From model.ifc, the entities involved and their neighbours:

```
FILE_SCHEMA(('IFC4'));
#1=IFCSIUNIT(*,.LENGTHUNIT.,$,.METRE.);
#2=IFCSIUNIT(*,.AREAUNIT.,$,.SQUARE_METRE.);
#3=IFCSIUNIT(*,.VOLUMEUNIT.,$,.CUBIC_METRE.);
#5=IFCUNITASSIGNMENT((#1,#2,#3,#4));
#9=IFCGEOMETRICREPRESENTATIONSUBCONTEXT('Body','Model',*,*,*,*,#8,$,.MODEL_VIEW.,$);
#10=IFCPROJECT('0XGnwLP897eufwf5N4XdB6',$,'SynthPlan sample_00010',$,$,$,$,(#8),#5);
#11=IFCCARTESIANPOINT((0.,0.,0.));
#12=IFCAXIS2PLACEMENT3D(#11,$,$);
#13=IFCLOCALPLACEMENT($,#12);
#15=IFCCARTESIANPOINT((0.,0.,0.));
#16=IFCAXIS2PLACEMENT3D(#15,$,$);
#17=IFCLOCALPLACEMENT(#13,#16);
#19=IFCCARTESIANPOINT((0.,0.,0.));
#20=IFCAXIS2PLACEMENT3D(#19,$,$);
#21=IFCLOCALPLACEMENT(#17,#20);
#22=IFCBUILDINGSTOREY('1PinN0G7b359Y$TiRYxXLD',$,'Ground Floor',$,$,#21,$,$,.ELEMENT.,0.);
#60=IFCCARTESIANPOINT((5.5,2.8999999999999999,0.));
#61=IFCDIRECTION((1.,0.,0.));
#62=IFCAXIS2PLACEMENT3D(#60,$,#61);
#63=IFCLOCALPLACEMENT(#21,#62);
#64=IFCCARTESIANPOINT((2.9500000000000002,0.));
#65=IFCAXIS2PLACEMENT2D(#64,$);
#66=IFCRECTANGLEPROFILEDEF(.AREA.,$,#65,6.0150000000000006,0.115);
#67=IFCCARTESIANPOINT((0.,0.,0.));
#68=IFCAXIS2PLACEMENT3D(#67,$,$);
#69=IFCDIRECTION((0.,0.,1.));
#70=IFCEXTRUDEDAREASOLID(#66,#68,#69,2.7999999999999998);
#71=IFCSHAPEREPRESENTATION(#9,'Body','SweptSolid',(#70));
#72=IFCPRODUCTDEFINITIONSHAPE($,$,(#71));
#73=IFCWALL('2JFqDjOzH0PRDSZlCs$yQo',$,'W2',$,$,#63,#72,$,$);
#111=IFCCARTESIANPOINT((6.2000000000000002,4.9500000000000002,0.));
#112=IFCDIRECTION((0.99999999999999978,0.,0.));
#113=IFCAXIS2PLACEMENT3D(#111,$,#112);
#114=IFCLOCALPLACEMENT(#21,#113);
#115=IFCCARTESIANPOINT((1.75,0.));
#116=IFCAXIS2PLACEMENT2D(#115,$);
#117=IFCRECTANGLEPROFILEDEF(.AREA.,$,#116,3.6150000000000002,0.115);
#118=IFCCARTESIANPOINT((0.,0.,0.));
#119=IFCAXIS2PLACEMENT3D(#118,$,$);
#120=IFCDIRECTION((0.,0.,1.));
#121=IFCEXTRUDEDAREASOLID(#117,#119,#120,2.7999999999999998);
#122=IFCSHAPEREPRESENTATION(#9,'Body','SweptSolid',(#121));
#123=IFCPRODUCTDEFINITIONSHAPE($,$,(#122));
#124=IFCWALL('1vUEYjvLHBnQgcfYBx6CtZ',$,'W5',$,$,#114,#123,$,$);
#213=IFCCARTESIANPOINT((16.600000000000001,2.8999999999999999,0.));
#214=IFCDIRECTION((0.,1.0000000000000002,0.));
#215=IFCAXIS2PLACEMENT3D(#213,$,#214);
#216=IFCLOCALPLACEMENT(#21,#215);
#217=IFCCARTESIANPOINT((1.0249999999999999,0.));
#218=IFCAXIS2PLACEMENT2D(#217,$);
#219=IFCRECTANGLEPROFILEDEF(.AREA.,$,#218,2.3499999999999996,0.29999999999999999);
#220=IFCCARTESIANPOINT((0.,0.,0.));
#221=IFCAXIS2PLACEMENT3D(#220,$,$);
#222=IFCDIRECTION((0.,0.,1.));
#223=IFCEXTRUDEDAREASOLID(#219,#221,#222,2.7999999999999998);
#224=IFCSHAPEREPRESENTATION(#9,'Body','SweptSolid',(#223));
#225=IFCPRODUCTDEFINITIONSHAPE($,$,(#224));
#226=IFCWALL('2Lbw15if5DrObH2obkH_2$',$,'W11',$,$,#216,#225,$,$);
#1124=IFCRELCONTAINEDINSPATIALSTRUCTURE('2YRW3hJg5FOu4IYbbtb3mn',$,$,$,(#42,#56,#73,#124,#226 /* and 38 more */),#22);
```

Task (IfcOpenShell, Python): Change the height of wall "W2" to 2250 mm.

```python
import ifcopenshell
import ifcopenshell.geom
import ifcopenshell.util.representation
import ifcopenshell.util.shape
import ifcopenshell.util.unit

model = ifcopenshell.open("model.ifc")
unit_scale = ifcopenshell.util.unit.calculate_unit_scale(model)
settings = ifcopenshell.geom.settings()


def volume(element):
    """Net volume in cubic metres, openings subtracted."""
    shape = ifcopenshell.geom.create_shape(settings, element)
    return ifcopenshell.util.shape.get_volume(shape.geometry)


wall = model.by_guid("2JFqDjOzH0PRDSZlCs$yQo")
before = volume(wall)

body = ifcopenshell.util.representation.get_representation(wall, "Model", "Body")
solid = body.Items[0]
old_height = solid.Depth
solid.Depth = 2.25 / unit_scale
after = volume(wall)

print(f"height {old_height:g} -> {solid.Depth:g}, volume {before:.3f} -> {after:.3f} m3")

model.write("model_v2.ifc")
```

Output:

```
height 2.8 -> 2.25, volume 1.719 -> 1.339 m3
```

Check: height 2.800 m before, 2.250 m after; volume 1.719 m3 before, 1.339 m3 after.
